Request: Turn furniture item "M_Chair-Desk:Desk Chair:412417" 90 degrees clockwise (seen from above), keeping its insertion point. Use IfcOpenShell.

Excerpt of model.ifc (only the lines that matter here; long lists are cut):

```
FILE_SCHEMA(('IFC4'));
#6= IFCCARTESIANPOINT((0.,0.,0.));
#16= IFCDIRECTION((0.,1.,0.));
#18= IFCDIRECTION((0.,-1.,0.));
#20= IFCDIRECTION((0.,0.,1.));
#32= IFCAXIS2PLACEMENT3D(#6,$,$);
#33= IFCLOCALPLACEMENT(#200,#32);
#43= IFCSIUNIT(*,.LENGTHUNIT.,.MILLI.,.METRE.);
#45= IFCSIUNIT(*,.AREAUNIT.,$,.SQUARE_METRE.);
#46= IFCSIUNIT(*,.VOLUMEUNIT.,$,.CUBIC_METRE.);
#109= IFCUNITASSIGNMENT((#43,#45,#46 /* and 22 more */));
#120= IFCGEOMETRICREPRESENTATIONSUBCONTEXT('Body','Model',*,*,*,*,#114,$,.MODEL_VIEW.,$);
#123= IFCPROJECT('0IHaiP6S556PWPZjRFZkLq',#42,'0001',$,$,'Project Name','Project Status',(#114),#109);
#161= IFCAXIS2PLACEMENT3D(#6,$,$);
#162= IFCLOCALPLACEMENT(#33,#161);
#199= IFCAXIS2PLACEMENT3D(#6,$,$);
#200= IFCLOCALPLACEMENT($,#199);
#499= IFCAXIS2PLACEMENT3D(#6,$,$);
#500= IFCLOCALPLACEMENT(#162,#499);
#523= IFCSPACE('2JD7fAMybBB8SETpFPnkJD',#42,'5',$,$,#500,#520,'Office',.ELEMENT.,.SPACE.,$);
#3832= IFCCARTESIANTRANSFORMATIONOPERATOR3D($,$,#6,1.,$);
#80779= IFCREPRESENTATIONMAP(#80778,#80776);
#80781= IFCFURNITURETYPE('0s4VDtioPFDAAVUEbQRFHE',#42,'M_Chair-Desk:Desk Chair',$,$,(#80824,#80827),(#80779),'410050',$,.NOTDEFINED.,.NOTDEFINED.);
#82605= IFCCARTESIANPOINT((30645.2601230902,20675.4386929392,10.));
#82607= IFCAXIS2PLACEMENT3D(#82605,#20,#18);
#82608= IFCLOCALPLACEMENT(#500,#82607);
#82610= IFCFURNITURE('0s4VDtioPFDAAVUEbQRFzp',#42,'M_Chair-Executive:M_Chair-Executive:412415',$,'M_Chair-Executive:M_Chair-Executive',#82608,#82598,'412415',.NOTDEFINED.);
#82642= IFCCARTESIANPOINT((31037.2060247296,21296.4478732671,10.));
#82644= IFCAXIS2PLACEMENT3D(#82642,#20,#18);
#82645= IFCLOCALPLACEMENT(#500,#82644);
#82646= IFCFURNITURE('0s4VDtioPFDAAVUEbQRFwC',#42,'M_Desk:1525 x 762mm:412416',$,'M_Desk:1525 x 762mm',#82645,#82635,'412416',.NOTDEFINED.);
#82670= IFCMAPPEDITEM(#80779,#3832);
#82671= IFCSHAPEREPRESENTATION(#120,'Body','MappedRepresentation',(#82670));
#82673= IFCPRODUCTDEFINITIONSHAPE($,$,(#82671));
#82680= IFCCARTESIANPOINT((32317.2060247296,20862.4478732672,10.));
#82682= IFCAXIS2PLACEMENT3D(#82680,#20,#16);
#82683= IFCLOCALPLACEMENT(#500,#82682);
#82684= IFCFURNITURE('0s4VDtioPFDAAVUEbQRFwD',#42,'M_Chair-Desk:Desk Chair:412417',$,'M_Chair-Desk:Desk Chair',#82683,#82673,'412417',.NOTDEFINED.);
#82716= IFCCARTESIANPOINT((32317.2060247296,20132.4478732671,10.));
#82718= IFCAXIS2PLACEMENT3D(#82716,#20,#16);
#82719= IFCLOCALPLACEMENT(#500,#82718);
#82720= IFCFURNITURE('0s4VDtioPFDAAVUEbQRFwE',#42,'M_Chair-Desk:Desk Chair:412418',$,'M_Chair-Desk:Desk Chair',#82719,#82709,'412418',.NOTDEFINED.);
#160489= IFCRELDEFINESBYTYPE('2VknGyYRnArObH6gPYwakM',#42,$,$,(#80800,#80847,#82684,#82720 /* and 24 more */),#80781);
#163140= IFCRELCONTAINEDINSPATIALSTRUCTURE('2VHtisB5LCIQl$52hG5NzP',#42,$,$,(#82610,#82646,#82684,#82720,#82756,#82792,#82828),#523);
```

```python
import ifcopenshell
import ifcopenshell.api.geometry
import ifcopenshell.util.placement

model = ifcopenshell.open("model.ifc")

item = model.by_id(82684)
matrix = ifcopenshell.util.placement.get_local_placement(item.ObjectPlacement)
matrix = matrix @ ifcopenshell.util.placement.rotation(-90, "Z")
ifcopenshell.api.geometry.edit_object_placement(model, product=item, matrix=matrix, is_si=False)

print(ifcopenshell.util.placement.get_local_placement(item.ObjectPlacement).round(3) + 0.0)

model.write("model_edited.ifc")
```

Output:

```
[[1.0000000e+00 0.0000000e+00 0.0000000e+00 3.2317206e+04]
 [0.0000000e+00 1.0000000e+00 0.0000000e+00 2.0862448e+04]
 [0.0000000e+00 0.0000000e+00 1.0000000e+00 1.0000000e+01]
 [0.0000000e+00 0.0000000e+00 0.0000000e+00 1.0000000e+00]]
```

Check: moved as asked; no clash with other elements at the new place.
